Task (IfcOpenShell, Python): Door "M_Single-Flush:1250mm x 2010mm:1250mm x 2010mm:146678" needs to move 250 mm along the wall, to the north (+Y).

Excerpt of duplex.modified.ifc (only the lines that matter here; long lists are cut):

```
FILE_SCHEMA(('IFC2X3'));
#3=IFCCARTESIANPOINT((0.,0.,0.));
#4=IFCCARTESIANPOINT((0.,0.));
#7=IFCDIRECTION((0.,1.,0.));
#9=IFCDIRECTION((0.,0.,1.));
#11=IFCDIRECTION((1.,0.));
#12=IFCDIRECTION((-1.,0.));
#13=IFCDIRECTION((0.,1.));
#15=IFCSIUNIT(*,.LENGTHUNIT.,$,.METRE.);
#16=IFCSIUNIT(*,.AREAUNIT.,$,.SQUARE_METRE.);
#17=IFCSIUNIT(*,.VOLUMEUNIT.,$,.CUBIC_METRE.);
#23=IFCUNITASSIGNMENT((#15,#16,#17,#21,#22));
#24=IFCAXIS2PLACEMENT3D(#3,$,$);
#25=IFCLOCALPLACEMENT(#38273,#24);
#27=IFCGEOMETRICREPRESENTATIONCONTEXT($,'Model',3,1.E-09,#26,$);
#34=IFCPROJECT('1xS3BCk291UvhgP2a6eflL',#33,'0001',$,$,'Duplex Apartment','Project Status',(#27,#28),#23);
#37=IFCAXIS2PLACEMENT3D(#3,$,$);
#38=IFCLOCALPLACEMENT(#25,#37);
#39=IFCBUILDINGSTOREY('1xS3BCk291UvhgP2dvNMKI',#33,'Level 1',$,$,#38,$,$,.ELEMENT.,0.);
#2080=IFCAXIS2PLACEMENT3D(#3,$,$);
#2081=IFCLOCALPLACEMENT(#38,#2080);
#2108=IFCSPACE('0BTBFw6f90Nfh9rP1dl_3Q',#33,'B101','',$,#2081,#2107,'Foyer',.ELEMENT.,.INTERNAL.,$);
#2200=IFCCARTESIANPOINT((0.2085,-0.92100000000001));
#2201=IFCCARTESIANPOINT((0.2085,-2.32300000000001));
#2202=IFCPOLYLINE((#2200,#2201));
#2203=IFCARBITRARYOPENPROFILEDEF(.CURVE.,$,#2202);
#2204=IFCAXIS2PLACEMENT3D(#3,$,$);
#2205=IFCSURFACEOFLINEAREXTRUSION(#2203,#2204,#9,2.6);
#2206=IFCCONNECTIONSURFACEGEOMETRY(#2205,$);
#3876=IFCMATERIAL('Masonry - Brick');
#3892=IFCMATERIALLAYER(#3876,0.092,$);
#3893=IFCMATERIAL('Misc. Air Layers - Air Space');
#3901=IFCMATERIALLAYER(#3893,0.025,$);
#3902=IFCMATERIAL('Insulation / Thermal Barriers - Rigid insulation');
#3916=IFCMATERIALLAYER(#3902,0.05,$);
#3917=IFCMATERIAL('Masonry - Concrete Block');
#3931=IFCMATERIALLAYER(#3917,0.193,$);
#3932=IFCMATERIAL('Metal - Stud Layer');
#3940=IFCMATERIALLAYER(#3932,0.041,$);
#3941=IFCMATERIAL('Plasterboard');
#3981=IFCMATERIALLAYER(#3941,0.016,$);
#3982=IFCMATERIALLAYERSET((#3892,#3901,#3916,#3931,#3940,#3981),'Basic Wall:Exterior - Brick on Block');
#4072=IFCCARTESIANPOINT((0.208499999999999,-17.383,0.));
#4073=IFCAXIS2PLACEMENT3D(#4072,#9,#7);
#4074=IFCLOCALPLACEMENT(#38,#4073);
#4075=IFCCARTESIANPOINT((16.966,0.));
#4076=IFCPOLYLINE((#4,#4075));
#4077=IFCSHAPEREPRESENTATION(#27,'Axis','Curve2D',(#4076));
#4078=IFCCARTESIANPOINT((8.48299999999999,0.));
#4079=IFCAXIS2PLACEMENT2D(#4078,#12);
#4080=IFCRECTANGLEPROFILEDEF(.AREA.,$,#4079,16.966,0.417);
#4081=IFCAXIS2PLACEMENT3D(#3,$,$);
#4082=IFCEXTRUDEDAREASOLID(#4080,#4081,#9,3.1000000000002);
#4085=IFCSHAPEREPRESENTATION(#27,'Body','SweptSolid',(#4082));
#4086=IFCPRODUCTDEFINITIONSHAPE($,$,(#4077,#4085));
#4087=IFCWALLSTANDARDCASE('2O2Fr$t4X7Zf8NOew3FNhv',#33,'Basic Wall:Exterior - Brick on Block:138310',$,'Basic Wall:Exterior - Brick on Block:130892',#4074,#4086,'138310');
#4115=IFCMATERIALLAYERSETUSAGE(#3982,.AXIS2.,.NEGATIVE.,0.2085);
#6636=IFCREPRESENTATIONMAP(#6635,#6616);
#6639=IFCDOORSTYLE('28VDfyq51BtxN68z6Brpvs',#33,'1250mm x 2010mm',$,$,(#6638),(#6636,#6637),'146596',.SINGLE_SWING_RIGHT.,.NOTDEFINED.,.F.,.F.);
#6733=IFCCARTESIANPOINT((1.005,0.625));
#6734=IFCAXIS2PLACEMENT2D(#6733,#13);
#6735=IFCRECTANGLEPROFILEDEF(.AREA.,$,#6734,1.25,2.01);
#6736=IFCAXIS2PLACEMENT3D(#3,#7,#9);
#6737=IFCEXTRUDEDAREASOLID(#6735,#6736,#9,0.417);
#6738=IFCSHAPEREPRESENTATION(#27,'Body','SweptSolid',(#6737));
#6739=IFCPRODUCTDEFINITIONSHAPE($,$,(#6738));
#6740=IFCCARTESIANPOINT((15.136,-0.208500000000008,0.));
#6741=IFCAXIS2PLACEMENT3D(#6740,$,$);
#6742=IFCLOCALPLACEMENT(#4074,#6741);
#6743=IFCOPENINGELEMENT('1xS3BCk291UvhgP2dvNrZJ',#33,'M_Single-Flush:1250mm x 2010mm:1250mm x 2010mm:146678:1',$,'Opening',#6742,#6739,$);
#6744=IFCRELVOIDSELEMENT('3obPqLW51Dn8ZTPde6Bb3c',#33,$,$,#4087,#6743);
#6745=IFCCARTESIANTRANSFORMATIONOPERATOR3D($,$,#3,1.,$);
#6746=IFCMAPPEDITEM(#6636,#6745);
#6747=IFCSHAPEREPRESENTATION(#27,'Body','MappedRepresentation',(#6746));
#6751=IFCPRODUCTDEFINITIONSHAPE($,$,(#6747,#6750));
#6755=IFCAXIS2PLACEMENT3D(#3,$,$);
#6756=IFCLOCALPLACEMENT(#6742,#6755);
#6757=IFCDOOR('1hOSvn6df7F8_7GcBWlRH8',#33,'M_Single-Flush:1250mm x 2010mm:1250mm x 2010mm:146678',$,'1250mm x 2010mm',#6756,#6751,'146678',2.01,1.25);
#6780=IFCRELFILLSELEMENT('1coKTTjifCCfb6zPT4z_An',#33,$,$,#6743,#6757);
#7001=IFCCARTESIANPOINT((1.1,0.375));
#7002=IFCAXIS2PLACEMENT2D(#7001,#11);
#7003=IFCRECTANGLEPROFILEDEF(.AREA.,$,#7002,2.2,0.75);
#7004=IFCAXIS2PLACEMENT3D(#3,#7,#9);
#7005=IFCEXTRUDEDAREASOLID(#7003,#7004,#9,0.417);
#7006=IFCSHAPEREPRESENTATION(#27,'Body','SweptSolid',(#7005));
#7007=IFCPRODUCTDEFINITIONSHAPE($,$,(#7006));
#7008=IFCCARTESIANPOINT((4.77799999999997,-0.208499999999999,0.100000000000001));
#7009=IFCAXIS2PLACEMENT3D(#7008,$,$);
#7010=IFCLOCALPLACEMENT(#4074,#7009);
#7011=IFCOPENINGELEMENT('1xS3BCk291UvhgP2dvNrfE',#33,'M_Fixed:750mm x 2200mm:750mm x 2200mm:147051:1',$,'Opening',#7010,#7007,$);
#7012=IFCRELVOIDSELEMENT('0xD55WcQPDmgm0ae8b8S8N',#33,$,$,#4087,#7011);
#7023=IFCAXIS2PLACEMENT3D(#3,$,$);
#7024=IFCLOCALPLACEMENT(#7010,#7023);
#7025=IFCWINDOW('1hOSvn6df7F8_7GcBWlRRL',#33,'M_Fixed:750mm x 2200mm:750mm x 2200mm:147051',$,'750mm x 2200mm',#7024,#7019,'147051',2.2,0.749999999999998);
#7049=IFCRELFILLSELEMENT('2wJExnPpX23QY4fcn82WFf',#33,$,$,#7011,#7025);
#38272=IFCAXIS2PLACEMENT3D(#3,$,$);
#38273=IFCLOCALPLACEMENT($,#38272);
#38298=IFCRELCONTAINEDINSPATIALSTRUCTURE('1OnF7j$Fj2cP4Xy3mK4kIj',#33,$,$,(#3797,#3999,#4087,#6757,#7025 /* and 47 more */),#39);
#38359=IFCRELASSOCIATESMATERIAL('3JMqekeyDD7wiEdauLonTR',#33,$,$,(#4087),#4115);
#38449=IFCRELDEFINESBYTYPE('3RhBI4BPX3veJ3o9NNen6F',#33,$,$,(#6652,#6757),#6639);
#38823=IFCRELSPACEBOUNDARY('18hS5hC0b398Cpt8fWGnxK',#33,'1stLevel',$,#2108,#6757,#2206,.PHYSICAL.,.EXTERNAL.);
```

```python
import numpy as np
import ifcopenshell
import ifcopenshell.api.geometry
import ifcopenshell.util.placement

model = ifcopenshell.open("duplex.modified.ifc")

door = model.by_id(6757)
opening = door.FillsVoids[0].RelatingOpeningElement
wall = opening.VoidsElements[0].RelatingBuildingElement

wall_matrix = ifcopenshell.util.placement.get_local_placement(wall.ObjectPlacement)
shift = wall_matrix[:3, 0] * 0.25
before = ifcopenshell.util.placement.get_local_placement(door.ObjectPlacement)[:3, 3].copy()

# The door is placed relative to its opening, so it follows when the opening moves.
matrix = ifcopenshell.util.placement.get_local_placement(opening.ObjectPlacement)
matrix[:3, 3] += shift
ifcopenshell.api.geometry.edit_object_placement(
    model, product=opening, matrix=matrix, is_si=False, should_transform_children=True
)

# Space boundary surfaces are stored in each space's coordinates; move them too.
for rel in door.ProvidesBoundaries:
    if not rel.ConnectionGeometry:
        continue
    surface = rel.ConnectionGeometry.SurfaceOnRelatingElement
    space_matrix = ifcopenshell.util.placement.get_local_placement(rel.RelatingSpace.ObjectPlacement)
    point = np.array(surface.Position.Location.Coordinates) + space_matrix[:3, :3].T @ shift
    surface.Position = model.createIfcAxis2Placement3D(
        model.createIfcCartesianPoint(point.tolist()), surface.Position.Axis, surface.Position.RefDirection
    )

after = ifcopenshell.util.placement.get_local_placement(door.ObjectPlacement)[:3, 3]
print("door moved by", (after - before).round(3) + 0.0)

model.write("duplex.modified_v2.ifc")
```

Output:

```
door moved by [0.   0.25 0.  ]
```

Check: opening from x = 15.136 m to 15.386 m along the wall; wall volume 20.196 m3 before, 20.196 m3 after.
